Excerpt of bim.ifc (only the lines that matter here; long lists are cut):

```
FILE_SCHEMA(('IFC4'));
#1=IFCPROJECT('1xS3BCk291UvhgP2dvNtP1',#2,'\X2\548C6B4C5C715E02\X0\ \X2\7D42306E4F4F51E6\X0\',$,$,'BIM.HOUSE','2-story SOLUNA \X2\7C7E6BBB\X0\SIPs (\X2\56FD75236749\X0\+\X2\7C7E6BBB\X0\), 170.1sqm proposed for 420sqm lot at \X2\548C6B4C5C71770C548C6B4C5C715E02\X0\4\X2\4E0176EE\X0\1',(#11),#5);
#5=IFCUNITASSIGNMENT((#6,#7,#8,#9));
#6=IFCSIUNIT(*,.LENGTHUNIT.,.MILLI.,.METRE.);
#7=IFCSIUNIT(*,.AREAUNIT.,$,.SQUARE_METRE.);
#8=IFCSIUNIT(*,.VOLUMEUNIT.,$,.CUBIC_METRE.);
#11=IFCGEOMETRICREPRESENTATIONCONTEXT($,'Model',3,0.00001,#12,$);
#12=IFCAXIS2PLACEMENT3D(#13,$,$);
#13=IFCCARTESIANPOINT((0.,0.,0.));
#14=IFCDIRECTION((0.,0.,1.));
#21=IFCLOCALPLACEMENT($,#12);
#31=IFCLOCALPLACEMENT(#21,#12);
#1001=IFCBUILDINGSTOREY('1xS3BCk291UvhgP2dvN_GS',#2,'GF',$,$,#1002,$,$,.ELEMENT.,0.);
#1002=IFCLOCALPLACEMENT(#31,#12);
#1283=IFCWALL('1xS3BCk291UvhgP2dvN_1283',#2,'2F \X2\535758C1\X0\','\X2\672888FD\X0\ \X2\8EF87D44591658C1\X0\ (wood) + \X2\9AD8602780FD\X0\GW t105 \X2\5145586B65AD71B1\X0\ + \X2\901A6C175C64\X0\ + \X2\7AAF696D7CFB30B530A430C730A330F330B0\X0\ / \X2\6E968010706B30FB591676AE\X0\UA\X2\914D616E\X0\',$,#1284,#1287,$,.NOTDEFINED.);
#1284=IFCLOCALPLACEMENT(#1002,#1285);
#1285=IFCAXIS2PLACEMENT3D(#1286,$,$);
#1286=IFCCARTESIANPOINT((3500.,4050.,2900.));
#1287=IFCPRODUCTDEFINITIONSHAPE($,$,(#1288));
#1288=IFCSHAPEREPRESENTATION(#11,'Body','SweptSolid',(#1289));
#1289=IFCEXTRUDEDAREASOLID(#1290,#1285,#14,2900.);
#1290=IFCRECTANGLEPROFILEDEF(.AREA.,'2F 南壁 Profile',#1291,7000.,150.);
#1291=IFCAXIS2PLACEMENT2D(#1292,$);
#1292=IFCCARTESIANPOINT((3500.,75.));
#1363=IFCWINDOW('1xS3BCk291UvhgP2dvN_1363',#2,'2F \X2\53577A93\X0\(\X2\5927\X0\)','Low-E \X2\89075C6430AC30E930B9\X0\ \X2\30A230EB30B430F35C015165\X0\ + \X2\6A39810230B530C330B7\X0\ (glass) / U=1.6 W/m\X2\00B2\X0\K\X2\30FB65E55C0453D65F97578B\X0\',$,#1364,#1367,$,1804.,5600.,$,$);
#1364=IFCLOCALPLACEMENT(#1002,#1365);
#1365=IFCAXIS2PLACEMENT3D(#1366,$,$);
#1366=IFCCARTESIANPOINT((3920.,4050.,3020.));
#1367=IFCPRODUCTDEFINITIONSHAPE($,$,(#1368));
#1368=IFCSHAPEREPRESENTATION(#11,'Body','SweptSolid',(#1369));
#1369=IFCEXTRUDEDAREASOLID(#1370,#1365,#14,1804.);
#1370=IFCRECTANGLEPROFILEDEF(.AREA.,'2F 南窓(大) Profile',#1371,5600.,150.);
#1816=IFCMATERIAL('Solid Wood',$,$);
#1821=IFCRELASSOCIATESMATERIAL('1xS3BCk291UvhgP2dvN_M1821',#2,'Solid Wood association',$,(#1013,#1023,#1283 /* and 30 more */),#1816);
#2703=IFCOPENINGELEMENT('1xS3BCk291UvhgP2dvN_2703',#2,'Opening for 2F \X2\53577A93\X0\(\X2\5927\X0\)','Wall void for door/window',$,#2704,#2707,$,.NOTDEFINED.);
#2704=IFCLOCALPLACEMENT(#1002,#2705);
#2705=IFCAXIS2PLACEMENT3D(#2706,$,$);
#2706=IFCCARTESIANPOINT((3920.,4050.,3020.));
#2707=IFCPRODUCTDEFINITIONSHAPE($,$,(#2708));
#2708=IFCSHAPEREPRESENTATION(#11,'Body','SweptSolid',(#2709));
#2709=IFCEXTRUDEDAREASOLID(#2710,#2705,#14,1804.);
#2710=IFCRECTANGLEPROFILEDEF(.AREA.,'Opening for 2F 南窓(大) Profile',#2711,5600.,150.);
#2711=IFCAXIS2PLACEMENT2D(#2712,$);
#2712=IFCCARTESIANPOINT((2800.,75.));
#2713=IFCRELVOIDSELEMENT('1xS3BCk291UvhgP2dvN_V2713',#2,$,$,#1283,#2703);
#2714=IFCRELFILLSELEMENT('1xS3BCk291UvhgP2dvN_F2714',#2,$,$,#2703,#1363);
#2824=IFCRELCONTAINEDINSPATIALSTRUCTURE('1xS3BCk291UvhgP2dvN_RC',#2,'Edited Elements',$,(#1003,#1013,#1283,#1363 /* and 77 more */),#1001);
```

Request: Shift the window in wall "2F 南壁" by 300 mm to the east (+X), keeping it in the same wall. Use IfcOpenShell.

```python
import ifcopenshell
import ifcopenshell.api.geometry
import ifcopenshell.util.placement
import ifcopenshell.util.unit

model = ifcopenshell.open("bim.ifc")
unit_scale = ifcopenshell.util.unit.calculate_unit_scale(model)

window = model.by_guid("1xS3BCk291UvhgP2dvN_1363")
opening = window.FillsVoids[0].RelatingOpeningElement
wall = opening.VoidsElements[0].RelatingBuildingElement

wall_matrix = ifcopenshell.util.placement.get_local_placement(wall.ObjectPlacement)
shift = wall_matrix[:3, 0] * 0.3 / unit_scale
before = ifcopenshell.util.placement.get_local_placement(window.ObjectPlacement)[:3, 3].copy()

# The window is not placed relative to its opening, so move both.
for product in (opening, window):
    matrix = ifcopenshell.util.placement.get_local_placement(product.ObjectPlacement)
    matrix[:3, 3] += shift
    ifcopenshell.api.geometry.edit_object_placement(model, product=product, matrix=matrix, is_si=False)

after = ifcopenshell.util.placement.get_local_placement(window.ObjectPlacement)[:3, 3]
print("window moved by", (after - before).round(3) + 0.0)

model.write("bim_rev.ifc")
```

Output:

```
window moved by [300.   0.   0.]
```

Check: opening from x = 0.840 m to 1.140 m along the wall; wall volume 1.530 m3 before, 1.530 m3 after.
